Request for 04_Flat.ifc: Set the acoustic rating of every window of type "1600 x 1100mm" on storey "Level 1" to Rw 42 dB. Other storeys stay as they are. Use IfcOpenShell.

First a look at what the model holds.

```python
import ifcopenshell
import ifcopenshell.util.element

model = ifcopenshell.open("04_Flat.ifc")
print(model.schema)
storey = next(s for s in model.by_type("IfcBuildingStorey") if s.Name == "Level 1")
windows = [e for e in ifcopenshell.util.element.get_decomposition(storey) if e.is_a("IfcWindow")]
seen = {}
for e in windows:
    element_type = ifcopenshell.util.element.get_type(e)
    key = (element_type.Name if element_type != e and element_type else None, ifcopenshell.util.element.get_pset(e, "Pset_WindowCommon", "AcousticRating"))
    seen[key] = seen.get(key, 0) + 1
for (name, value), count in sorted(seen.items(), key=str):
    print(count, "x", name, "|", value)
```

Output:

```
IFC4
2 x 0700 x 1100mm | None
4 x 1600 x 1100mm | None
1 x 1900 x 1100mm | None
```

```python
import ifcopenshell
import ifcopenshell.api.pset
import ifcopenshell.util.element

model = ifcopenshell.open("04_Flat.ifc")

storey = next(s for s in model.by_type("IfcBuildingStorey") if s.Name == "Level 1")
windows = [e for e in ifcopenshell.util.element.get_decomposition(storey) if e.is_a("IfcWindow")]

count = 0
for e in windows:
    element_type = ifcopenshell.util.element.get_type(e)
    if element_type in (None, e) or element_type.Name != "1600 x 1100mm":
        continue
    # add_pset returns the element's existing set when there is one.
    pset = ifcopenshell.api.pset.add_pset(model, product=e, name="Pset_WindowCommon")
    ifcopenshell.api.pset.edit_pset(model, pset=pset, properties={"AcousticRating": "Rw 42 dB"})
    count += 1

print(count, "windows updated")

model.write("04_Flat_updated.ifc")
```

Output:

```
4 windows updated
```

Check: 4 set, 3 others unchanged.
